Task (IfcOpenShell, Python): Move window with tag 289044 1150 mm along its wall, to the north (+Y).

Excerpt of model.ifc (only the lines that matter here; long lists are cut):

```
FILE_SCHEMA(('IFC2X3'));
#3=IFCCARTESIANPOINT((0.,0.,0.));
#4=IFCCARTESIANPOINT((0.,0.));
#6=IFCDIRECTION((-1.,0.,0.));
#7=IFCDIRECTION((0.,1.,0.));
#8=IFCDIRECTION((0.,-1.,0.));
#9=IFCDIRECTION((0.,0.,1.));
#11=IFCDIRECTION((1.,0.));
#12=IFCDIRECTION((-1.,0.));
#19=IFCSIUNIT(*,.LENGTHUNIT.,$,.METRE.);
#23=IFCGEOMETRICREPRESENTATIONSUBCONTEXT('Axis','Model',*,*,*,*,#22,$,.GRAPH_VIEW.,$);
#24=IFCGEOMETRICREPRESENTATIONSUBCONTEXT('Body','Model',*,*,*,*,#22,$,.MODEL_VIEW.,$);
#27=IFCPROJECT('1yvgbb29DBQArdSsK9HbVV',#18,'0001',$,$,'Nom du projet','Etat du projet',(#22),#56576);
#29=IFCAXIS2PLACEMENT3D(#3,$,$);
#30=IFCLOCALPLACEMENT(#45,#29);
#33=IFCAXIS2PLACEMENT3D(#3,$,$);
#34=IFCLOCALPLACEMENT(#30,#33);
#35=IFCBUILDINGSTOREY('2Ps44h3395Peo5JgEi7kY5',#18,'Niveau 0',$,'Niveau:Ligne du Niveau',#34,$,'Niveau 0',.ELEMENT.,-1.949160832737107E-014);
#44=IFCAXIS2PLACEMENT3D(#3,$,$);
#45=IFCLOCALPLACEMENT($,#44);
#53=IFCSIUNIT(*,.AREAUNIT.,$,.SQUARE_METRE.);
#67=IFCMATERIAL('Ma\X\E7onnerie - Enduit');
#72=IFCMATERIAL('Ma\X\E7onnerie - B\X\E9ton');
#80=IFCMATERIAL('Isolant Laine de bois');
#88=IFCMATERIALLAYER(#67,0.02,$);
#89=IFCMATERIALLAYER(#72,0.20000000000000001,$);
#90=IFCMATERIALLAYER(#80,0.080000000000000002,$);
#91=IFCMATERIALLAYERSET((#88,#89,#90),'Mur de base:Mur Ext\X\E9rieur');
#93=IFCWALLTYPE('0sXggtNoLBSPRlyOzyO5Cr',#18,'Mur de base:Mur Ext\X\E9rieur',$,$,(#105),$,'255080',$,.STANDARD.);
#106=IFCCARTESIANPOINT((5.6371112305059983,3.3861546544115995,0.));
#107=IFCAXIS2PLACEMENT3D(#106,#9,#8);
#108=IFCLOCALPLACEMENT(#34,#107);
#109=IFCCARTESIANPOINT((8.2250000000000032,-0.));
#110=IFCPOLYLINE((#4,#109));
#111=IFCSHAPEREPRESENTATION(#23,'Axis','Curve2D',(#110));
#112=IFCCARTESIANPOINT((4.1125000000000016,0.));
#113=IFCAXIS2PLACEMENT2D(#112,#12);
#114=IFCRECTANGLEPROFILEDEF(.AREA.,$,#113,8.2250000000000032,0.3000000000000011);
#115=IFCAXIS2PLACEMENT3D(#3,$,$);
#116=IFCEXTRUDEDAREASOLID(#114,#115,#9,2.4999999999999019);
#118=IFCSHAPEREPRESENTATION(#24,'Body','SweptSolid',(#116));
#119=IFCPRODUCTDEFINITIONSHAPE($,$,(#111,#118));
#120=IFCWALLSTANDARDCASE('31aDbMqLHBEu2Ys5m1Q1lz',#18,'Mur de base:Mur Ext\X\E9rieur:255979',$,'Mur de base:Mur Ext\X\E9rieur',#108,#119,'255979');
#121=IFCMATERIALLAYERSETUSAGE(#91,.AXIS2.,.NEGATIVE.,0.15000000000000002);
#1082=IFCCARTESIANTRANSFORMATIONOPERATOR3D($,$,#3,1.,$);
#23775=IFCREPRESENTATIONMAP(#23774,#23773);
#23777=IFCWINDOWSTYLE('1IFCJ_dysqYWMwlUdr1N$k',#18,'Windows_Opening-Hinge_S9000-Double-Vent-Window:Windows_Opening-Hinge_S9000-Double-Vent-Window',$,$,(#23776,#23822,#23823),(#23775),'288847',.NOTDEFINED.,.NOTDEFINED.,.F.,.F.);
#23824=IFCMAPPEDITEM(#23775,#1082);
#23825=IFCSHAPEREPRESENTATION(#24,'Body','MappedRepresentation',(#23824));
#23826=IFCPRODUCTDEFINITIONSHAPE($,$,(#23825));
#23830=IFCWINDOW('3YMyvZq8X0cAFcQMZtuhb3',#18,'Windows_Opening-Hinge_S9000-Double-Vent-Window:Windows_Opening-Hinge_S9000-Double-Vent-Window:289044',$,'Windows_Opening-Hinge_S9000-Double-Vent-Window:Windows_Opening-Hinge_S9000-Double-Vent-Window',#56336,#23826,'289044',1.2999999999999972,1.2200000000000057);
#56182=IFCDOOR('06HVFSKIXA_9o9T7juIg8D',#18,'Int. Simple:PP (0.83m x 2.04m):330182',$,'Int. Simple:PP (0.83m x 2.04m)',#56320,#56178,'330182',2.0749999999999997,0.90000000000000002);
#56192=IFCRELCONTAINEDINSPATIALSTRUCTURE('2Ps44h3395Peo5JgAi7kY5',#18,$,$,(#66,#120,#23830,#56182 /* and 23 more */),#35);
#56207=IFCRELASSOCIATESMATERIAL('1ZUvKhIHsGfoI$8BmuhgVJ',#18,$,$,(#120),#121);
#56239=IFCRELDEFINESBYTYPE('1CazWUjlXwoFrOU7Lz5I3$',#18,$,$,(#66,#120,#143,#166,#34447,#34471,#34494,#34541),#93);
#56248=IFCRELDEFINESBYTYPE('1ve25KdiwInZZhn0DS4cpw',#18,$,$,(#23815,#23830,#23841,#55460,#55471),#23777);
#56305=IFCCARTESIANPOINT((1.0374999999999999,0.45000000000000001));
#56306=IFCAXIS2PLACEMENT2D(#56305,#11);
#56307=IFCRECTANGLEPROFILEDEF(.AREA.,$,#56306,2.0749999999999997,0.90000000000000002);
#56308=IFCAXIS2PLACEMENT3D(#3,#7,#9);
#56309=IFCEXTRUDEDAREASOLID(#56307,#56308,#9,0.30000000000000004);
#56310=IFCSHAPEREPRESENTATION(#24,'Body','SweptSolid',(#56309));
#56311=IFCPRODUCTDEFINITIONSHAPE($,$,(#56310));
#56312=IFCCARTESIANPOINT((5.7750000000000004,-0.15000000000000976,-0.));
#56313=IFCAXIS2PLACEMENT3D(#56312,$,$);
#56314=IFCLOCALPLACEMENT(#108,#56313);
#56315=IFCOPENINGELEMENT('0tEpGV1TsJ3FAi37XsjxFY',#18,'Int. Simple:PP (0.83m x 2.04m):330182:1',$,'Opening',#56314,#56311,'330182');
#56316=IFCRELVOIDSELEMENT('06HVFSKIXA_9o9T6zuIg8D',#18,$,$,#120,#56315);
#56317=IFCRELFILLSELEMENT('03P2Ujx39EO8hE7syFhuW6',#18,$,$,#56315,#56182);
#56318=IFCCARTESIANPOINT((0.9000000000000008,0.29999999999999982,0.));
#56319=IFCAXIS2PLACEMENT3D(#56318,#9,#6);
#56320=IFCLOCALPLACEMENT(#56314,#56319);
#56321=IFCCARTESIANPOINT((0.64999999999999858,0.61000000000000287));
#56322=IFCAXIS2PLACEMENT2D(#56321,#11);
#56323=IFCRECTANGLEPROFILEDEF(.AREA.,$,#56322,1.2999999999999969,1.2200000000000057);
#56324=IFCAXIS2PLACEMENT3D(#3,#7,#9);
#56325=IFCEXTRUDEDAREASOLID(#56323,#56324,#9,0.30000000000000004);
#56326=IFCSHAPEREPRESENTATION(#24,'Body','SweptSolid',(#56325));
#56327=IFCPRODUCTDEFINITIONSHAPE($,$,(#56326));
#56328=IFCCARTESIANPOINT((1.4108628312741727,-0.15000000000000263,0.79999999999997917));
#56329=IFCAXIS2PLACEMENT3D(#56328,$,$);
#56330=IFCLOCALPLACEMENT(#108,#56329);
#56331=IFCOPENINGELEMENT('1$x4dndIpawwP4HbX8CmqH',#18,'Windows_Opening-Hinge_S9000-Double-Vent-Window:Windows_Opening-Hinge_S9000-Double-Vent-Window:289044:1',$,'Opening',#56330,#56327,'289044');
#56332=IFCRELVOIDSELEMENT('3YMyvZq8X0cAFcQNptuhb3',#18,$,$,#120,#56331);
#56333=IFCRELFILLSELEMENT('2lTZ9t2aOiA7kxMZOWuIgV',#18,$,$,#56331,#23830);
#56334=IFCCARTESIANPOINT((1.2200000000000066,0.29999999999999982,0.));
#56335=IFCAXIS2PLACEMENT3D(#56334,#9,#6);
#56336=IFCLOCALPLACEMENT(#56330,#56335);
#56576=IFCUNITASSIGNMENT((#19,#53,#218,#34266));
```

```python
import ifcopenshell
import ifcopenshell.api.geometry
import ifcopenshell.util.placement

model = ifcopenshell.open("model.ifc")

window = model.by_id(23830)
opening = window.FillsVoids[0].RelatingOpeningElement
wall = opening.VoidsElements[0].RelatingBuildingElement

wall_matrix = ifcopenshell.util.placement.get_local_placement(wall.ObjectPlacement)
shift = wall_matrix[:3, 0] * -1.15
before = ifcopenshell.util.placement.get_local_placement(window.ObjectPlacement)[:3, 3].copy()

# The window is placed relative to its opening, so it follows when the opening moves.
matrix = ifcopenshell.util.placement.get_local_placement(opening.ObjectPlacement)
matrix[:3, 3] += shift
ifcopenshell.api.geometry.edit_object_placement(
    model, product=opening, matrix=matrix, is_si=False, should_transform_children=True
)

after = ifcopenshell.util.placement.get_local_placement(window.ObjectPlacement)[:3, 3]
print("window moved by", (after - before).round(3) + 0.0)

model.write("model_v2.ifc")
```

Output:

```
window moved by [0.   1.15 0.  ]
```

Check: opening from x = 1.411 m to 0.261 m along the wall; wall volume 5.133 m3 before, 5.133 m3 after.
